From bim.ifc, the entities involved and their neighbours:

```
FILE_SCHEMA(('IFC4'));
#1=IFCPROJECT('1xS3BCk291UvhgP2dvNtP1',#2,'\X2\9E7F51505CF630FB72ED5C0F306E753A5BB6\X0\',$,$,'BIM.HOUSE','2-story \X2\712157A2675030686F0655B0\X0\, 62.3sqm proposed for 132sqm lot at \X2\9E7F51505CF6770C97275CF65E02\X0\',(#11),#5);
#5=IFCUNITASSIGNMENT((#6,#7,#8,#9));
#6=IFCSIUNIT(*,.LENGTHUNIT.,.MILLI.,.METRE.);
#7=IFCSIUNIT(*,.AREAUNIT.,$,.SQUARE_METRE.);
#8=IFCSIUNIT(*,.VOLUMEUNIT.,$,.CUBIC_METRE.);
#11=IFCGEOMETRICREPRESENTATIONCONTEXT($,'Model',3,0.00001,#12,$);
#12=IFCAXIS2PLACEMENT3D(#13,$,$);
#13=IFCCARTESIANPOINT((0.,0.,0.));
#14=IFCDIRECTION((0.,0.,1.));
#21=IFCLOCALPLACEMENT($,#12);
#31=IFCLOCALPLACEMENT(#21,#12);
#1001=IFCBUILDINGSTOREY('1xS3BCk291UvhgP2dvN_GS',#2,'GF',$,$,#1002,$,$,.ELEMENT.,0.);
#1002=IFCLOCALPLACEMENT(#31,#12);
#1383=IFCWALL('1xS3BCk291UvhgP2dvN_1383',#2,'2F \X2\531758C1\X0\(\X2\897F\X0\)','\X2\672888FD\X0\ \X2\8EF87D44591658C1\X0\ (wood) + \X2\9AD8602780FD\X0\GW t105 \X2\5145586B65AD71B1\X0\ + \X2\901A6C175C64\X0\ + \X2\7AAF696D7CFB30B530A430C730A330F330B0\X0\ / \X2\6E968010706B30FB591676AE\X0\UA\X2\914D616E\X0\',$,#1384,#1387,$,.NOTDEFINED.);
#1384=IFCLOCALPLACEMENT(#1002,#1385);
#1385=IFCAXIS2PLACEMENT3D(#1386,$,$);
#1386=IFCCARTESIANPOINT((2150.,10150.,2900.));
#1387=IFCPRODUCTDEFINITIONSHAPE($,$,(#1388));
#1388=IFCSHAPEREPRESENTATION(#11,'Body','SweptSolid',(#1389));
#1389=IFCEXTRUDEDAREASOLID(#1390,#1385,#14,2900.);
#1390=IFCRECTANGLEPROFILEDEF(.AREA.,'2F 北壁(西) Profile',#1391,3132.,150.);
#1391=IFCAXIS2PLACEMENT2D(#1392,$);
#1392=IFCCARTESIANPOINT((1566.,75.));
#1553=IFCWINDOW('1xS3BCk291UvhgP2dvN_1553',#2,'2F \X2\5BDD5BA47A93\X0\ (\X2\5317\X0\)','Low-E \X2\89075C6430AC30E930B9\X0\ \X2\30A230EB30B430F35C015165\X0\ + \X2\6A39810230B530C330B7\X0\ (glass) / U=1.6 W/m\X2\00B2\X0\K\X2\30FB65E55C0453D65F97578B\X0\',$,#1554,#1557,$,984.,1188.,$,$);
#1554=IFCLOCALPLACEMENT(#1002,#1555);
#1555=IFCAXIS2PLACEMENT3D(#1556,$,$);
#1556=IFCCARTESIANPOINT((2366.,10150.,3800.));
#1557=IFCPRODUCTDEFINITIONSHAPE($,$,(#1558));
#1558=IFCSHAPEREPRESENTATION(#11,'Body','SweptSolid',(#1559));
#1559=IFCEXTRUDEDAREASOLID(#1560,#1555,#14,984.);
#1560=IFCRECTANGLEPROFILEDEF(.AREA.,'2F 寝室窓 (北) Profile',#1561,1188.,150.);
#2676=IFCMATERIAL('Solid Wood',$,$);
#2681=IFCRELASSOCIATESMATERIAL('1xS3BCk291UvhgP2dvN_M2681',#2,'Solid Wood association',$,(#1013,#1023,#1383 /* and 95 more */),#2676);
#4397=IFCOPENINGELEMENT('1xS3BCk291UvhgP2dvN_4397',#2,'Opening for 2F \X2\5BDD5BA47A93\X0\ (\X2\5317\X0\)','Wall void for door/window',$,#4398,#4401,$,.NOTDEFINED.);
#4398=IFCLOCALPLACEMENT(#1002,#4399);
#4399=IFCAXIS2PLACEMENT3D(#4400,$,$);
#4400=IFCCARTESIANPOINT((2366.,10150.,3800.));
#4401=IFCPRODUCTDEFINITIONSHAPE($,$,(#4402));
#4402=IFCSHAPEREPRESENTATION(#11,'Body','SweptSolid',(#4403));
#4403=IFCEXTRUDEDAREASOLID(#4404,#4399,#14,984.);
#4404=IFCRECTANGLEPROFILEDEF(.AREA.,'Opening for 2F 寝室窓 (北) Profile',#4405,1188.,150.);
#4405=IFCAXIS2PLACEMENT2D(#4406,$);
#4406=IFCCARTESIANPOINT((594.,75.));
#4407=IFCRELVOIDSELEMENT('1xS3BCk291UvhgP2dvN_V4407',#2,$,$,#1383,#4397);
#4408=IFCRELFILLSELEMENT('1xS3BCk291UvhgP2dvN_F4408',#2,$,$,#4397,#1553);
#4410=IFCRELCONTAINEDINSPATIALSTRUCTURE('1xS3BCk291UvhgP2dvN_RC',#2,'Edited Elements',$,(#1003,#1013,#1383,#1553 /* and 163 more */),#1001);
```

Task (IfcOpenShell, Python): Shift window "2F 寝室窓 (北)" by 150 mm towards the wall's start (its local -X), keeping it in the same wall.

```python
import ifcopenshell
import ifcopenshell.api.geometry
import ifcopenshell.util.placement
import ifcopenshell.util.unit

model = ifcopenshell.open("bim.ifc")
unit_scale = ifcopenshell.util.unit.calculate_unit_scale(model)

window = model.by_guid("1xS3BCk291UvhgP2dvN_1553")
opening = window.FillsVoids[0].RelatingOpeningElement
wall = opening.VoidsElements[0].RelatingBuildingElement

wall_matrix = ifcopenshell.util.placement.get_local_placement(wall.ObjectPlacement)
shift = wall_matrix[:3, 0] * -0.15 / unit_scale
before = ifcopenshell.util.placement.get_local_placement(window.ObjectPlacement)[:3, 3].copy()

# The window is not placed relative to its opening, so move both.
for product in (opening, window):
    matrix = ifcopenshell.util.placement.get_local_placement(product.ObjectPlacement)
    matrix[:3, 3] += shift
    ifcopenshell.api.geometry.edit_object_placement(model, product=product, matrix=matrix, is_si=False)

after = ifcopenshell.util.placement.get_local_placement(window.ObjectPlacement)[:3, 3]
print("window moved by", (after - before).round(3) + 0.0)

model.write("bim_edited.ifc")
```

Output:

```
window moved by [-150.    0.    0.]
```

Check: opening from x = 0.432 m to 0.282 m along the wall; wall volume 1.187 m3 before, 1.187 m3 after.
